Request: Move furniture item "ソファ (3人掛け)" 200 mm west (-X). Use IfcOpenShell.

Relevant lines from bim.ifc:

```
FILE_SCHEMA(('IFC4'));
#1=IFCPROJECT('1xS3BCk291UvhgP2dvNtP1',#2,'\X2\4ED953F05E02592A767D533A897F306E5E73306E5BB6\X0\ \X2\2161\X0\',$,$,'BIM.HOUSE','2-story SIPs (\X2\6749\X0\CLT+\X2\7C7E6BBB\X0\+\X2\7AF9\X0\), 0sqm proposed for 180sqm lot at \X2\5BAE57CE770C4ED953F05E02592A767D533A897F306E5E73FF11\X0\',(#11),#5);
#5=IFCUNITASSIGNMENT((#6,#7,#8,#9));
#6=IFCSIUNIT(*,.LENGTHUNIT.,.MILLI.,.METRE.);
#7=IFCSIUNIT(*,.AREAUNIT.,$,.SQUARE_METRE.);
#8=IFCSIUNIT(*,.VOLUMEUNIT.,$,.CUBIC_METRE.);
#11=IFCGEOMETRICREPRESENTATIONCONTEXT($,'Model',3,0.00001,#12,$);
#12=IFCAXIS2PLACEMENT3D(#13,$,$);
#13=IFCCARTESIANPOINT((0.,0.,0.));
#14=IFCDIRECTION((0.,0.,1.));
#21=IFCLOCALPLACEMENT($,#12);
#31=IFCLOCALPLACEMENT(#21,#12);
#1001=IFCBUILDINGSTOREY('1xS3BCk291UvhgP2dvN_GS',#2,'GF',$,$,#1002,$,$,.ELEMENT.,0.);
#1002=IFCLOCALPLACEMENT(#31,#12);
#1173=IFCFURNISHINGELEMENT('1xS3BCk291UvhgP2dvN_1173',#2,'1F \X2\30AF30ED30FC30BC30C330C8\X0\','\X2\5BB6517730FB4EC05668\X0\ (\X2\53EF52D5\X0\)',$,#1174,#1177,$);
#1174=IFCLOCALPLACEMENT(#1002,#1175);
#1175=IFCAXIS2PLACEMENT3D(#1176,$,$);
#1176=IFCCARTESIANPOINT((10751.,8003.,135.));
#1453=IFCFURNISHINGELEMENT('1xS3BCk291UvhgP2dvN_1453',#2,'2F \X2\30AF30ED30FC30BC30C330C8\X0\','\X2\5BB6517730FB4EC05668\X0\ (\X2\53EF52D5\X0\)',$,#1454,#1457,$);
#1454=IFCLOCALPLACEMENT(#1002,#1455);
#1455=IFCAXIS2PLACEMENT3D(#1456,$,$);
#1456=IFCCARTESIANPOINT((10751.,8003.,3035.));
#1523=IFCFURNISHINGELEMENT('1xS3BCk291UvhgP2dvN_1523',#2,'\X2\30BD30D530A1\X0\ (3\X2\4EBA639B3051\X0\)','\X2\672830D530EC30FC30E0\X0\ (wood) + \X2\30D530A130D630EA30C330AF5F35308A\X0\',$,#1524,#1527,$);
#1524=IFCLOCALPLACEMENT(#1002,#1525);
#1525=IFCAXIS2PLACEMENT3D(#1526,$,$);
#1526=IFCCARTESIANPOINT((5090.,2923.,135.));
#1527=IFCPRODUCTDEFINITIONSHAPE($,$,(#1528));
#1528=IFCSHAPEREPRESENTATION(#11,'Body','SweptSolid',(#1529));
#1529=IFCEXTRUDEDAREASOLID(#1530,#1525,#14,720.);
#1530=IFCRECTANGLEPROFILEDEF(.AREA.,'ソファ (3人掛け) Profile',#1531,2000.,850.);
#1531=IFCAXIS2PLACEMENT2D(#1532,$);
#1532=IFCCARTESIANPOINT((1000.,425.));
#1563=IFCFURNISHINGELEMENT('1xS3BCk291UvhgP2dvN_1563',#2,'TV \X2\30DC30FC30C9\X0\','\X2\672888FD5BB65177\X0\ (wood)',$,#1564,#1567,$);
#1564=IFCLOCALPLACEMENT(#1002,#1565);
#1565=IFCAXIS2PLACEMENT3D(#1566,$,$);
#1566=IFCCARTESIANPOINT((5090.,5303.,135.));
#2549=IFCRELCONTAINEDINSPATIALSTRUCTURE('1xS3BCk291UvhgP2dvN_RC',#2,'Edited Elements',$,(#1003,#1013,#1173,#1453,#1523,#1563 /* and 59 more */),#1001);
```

```python
import ifcopenshell
import ifcopenshell.api.geometry
import ifcopenshell.util.placement

model = ifcopenshell.open("bim.ifc")

item = model.by_id(1523)
matrix = ifcopenshell.util.placement.get_local_placement(item.ObjectPlacement)
matrix[0, 3] -= 200.0
ifcopenshell.api.geometry.edit_object_placement(model, product=item, matrix=matrix, is_si=False)

print(ifcopenshell.util.placement.get_local_placement(item.ObjectPlacement).round(3) + 0.0)

model.write("bim_updated.ifc")
```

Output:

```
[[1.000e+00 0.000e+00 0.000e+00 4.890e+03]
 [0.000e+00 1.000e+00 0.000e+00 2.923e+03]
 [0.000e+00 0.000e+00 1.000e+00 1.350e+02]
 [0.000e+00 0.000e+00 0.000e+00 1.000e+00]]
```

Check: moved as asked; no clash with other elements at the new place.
